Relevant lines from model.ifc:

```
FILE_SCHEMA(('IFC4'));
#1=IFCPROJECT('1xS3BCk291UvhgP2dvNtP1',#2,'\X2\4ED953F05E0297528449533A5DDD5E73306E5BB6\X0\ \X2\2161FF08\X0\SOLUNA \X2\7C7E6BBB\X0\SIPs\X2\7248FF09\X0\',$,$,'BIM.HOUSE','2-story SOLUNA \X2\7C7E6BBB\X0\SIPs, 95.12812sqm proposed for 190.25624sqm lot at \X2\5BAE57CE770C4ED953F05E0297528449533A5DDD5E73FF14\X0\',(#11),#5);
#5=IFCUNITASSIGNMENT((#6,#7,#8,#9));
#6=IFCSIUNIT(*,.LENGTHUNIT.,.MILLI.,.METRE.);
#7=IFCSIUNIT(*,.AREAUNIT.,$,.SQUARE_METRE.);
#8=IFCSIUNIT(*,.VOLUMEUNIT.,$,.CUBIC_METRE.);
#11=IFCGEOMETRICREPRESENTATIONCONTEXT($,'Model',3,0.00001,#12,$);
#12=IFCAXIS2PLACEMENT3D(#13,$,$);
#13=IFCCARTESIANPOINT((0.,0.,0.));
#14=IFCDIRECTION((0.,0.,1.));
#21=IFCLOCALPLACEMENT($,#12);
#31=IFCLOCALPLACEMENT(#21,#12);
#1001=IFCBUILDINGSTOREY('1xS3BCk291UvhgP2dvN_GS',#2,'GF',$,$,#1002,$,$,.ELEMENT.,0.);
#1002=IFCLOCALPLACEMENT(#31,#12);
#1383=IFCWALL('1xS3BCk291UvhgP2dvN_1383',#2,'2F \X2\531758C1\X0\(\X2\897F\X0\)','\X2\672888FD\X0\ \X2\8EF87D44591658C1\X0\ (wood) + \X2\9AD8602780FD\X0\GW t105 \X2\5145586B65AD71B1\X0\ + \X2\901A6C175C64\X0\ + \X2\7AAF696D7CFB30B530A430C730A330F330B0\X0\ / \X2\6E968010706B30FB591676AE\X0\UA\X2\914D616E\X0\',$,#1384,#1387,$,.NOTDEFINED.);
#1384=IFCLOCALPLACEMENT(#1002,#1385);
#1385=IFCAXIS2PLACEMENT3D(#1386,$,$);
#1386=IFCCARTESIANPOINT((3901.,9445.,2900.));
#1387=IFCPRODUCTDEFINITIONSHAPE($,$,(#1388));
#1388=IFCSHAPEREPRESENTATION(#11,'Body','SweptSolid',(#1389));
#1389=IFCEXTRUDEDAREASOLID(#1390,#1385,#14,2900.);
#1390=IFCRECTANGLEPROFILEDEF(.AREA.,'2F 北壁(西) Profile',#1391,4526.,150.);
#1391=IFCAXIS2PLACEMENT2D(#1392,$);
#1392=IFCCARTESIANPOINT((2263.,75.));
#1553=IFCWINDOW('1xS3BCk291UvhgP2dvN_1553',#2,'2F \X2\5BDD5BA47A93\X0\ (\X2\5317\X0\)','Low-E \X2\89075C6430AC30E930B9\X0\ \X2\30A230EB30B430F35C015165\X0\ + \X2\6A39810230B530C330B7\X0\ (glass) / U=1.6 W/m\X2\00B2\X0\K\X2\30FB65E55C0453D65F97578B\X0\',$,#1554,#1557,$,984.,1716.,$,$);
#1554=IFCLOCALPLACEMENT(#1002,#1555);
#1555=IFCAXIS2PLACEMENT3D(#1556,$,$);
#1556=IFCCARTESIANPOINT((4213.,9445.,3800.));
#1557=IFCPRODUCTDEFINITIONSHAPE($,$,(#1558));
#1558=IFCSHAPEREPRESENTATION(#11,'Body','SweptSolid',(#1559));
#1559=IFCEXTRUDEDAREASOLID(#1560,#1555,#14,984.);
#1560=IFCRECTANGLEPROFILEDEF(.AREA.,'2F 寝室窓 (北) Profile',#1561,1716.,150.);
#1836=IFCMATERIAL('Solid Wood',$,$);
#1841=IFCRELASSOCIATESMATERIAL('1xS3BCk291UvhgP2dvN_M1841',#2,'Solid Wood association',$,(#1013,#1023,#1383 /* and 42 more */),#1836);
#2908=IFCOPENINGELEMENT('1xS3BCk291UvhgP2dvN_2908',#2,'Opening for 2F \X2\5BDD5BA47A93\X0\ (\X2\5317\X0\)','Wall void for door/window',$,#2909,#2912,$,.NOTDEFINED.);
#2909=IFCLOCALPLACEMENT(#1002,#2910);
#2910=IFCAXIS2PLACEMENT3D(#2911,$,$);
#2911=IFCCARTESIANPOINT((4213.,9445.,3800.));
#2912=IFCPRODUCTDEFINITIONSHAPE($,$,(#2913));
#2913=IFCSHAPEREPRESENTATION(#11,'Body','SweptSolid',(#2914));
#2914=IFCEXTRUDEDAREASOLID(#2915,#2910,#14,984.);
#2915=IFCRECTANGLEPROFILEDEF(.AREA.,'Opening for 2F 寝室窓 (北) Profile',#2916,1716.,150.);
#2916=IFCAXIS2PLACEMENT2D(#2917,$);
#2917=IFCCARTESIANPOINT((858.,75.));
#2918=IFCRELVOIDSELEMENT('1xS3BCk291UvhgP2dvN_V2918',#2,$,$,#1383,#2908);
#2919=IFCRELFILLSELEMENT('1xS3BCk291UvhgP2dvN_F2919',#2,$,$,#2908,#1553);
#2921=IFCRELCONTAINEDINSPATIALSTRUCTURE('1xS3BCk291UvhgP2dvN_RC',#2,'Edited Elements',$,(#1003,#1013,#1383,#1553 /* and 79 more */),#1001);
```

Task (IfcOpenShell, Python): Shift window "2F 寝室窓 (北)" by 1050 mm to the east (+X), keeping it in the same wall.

```python
import ifcopenshell
import ifcopenshell.api.geometry
import ifcopenshell.util.placement
import ifcopenshell.util.unit

model = ifcopenshell.open("model.ifc")
unit_scale = ifcopenshell.util.unit.calculate_unit_scale(model)

window = model.by_guid("1xS3BCk291UvhgP2dvN_1553")
opening = window.FillsVoids[0].RelatingOpeningElement
wall = opening.VoidsElements[0].RelatingBuildingElement

wall_matrix = ifcopenshell.util.placement.get_local_placement(wall.ObjectPlacement)
shift = wall_matrix[:3, 0] * 1.05 / unit_scale
before = ifcopenshell.util.placement.get_local_placement(window.ObjectPlacement)[:3, 3].copy()

# The window is not placed relative to its opening, so move both.
for product in (opening, window):
    matrix = ifcopenshell.util.placement.get_local_placement(product.ObjectPlacement)
    matrix[:3, 3] += shift
    ifcopenshell.api.geometry.edit_object_placement(model, product=product, matrix=matrix, is_si=False)

after = ifcopenshell.util.placement.get_local_placement(window.ObjectPlacement)[:3, 3]
print("window moved by", (after - before).round(3) + 0.0)

model.write("model_updated.ifc")
```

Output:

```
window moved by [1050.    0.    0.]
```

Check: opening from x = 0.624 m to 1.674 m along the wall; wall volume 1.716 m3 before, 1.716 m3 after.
